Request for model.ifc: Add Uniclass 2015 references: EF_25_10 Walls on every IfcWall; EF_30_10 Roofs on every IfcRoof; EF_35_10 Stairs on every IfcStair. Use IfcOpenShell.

First a look at what the model holds.

```python
import ifcopenshell

model = ifcopenshell.open("model.ifc")
print(model.schema)
print("classifications:", [c.Name for c in model.by_type("IfcClassification")])
for ifc_class in ("IfcDoor", "IfcRoof", "IfcStair", "IfcWall", "IfcWindow"):
    print(ifc_class, len(model.by_type(ifc_class)))
```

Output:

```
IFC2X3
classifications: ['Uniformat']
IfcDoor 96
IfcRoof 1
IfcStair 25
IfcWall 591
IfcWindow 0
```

```python
import ifcopenshell
import ifcopenshell.api.classification

model = ifcopenshell.open("model.ifc")

# IFC2X3 requires Source and Edition and has no link from the project to the system.
system = model.create_entity("IfcClassification", Source="NBS", Edition="2015", Name="Uniclass 2015")

codes = {
    "IfcWall": ("EF_25_10", "Walls"),
    "IfcRoof": ("EF_30_10", "Roofs"),
    "IfcStair": ("EF_35_10", "Stairs"),
}
for ifc_class, (code, name) in codes.items():
    products = model.by_type(ifc_class)
    ifcopenshell.api.classification.add_reference(
        model, products=products, classification=system, identification=code, name=name
    )
    print(code, len(products))

model.write("model_v2.ifc")
```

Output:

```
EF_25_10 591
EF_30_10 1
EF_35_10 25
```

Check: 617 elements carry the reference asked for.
